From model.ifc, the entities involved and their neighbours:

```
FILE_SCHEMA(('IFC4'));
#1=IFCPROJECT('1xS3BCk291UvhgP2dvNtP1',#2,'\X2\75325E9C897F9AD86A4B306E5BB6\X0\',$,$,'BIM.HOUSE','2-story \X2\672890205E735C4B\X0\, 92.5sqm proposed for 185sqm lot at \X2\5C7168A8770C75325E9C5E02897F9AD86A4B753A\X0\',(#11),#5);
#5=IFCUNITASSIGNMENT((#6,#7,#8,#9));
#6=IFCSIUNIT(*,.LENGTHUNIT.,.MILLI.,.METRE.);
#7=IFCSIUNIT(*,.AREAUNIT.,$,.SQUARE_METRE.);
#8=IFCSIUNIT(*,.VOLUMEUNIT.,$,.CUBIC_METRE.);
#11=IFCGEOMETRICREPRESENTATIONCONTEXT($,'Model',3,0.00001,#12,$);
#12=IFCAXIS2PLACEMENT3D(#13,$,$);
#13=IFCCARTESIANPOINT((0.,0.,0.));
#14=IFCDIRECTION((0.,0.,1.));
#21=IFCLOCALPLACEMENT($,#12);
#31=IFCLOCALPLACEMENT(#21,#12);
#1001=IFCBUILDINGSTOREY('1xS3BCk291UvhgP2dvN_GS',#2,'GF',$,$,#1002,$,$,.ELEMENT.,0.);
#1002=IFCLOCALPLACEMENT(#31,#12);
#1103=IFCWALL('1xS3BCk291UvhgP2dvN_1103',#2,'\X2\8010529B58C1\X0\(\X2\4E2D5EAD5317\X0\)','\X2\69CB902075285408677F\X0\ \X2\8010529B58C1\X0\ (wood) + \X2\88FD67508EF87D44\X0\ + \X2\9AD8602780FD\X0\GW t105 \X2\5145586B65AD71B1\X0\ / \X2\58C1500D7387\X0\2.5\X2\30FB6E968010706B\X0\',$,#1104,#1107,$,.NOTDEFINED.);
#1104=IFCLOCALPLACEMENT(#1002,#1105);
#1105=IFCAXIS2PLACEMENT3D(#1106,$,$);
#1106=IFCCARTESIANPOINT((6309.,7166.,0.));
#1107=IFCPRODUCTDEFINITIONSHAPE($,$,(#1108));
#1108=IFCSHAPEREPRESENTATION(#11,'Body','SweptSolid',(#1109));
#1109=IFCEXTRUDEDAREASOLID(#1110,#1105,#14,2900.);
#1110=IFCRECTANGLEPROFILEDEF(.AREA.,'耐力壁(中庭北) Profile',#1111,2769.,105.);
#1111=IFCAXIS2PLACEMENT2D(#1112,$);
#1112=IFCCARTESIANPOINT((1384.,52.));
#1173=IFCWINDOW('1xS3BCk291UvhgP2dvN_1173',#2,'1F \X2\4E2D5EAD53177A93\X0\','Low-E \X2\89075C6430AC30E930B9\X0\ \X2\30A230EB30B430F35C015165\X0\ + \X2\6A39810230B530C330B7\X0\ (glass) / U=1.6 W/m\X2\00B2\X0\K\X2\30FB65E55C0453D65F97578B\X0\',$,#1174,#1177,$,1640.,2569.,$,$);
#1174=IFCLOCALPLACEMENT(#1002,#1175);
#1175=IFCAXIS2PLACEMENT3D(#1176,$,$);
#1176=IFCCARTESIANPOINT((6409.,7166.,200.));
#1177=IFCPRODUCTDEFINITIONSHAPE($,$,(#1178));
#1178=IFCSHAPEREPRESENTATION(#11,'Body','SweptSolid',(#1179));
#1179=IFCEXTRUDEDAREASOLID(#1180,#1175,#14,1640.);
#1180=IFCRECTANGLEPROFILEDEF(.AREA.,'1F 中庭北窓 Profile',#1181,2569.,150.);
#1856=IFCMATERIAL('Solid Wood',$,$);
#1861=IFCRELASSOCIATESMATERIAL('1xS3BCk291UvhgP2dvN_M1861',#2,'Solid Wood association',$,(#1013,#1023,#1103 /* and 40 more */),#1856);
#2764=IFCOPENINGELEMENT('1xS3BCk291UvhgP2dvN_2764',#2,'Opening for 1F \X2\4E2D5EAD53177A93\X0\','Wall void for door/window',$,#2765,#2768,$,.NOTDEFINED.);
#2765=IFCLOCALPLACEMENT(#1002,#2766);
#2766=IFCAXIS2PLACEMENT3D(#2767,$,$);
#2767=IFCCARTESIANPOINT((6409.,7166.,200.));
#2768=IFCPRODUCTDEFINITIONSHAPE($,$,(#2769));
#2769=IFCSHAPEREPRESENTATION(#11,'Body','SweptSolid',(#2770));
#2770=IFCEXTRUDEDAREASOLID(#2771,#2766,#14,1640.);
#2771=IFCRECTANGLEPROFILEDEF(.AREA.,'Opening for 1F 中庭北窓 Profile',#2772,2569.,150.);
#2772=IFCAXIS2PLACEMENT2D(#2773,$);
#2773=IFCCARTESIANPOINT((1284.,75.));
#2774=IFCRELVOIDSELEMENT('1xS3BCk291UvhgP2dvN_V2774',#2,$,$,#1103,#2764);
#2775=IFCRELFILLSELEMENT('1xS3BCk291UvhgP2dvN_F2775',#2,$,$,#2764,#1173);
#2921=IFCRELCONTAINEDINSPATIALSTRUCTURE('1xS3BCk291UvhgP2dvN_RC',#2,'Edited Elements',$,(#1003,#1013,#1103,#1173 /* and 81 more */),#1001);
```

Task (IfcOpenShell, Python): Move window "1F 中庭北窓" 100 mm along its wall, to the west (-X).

```python
import ifcopenshell
import ifcopenshell.api.geometry
import ifcopenshell.util.placement
import ifcopenshell.util.unit

model = ifcopenshell.open("model.ifc")
unit_scale = ifcopenshell.util.unit.calculate_unit_scale(model)

window = model.by_id(1173)
opening = window.FillsVoids[0].RelatingOpeningElement
wall = opening.VoidsElements[0].RelatingBuildingElement

wall_matrix = ifcopenshell.util.placement.get_local_placement(wall.ObjectPlacement)
shift = wall_matrix[:3, 0] * -0.1 / unit_scale
before = ifcopenshell.util.placement.get_local_placement(window.ObjectPlacement)[:3, 3].copy()

# The window is not placed relative to its opening, so move both.
for product in (opening, window):
    matrix = ifcopenshell.util.placement.get_local_placement(product.ObjectPlacement)
    matrix[:3, 3] += shift
    ifcopenshell.api.geometry.edit_object_placement(model, product=product, matrix=matrix, is_si=False)

after = ifcopenshell.util.placement.get_local_placement(window.ObjectPlacement)[:3, 3]
print("window moved by", (after - before).round(3) + 0.0)

model.write("model_v2.ifc")
```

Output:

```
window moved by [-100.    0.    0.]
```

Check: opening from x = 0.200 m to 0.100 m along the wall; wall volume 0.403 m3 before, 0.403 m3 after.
